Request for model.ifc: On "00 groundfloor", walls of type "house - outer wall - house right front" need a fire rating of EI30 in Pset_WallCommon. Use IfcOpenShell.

First a look at what the model holds.

```python
import ifcopenshell
import ifcopenshell.util.element

model = ifcopenshell.open("model.ifc")
print(model.schema)
storey = next(s for s in model.by_type("IfcBuildingStorey") if s.Name == "00 groundfloor")
walls = [e for e in ifcopenshell.util.element.get_decomposition(storey) if e.is_a("IfcWall")]
seen = {}
for e in walls:
    element_type = ifcopenshell.util.element.get_type(e)
    key = (element_type.Name if element_type != e and element_type else None, ifcopenshell.util.element.get_pset(e, "Pset_WallCommon", "FireRating"))
    seen[key] = seen.get(key, 0) + 1
for (name, value), count in sorted(seen.items(), key=str):
    print(count, "x", name, "|", value)
```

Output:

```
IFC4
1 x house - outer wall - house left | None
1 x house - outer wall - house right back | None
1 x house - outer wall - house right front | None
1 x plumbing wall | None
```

```python
import ifcopenshell
import ifcopenshell.api.pset
import ifcopenshell.util.element

model = ifcopenshell.open("model.ifc")

storey = next(s for s in model.by_type("IfcBuildingStorey") if s.Name == "00 groundfloor")
walls = [e for e in ifcopenshell.util.element.get_decomposition(storey) if e.is_a("IfcWall")]

count = 0
for e in walls:
    element_type = ifcopenshell.util.element.get_type(e)
    if element_type in (None, e) or element_type.Name != "house - outer wall - house right front":
        continue
    # add_pset returns the element's existing set when there is one.
    pset = ifcopenshell.api.pset.add_pset(model, product=e, name="Pset_WallCommon")
    ifcopenshell.api.pset.edit_pset(model, pset=pset, properties={"FireRating": "EI30"})
    count += 1

print(count, "walls updated")

model.write("model_rev.ifc")
```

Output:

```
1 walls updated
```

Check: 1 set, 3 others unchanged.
